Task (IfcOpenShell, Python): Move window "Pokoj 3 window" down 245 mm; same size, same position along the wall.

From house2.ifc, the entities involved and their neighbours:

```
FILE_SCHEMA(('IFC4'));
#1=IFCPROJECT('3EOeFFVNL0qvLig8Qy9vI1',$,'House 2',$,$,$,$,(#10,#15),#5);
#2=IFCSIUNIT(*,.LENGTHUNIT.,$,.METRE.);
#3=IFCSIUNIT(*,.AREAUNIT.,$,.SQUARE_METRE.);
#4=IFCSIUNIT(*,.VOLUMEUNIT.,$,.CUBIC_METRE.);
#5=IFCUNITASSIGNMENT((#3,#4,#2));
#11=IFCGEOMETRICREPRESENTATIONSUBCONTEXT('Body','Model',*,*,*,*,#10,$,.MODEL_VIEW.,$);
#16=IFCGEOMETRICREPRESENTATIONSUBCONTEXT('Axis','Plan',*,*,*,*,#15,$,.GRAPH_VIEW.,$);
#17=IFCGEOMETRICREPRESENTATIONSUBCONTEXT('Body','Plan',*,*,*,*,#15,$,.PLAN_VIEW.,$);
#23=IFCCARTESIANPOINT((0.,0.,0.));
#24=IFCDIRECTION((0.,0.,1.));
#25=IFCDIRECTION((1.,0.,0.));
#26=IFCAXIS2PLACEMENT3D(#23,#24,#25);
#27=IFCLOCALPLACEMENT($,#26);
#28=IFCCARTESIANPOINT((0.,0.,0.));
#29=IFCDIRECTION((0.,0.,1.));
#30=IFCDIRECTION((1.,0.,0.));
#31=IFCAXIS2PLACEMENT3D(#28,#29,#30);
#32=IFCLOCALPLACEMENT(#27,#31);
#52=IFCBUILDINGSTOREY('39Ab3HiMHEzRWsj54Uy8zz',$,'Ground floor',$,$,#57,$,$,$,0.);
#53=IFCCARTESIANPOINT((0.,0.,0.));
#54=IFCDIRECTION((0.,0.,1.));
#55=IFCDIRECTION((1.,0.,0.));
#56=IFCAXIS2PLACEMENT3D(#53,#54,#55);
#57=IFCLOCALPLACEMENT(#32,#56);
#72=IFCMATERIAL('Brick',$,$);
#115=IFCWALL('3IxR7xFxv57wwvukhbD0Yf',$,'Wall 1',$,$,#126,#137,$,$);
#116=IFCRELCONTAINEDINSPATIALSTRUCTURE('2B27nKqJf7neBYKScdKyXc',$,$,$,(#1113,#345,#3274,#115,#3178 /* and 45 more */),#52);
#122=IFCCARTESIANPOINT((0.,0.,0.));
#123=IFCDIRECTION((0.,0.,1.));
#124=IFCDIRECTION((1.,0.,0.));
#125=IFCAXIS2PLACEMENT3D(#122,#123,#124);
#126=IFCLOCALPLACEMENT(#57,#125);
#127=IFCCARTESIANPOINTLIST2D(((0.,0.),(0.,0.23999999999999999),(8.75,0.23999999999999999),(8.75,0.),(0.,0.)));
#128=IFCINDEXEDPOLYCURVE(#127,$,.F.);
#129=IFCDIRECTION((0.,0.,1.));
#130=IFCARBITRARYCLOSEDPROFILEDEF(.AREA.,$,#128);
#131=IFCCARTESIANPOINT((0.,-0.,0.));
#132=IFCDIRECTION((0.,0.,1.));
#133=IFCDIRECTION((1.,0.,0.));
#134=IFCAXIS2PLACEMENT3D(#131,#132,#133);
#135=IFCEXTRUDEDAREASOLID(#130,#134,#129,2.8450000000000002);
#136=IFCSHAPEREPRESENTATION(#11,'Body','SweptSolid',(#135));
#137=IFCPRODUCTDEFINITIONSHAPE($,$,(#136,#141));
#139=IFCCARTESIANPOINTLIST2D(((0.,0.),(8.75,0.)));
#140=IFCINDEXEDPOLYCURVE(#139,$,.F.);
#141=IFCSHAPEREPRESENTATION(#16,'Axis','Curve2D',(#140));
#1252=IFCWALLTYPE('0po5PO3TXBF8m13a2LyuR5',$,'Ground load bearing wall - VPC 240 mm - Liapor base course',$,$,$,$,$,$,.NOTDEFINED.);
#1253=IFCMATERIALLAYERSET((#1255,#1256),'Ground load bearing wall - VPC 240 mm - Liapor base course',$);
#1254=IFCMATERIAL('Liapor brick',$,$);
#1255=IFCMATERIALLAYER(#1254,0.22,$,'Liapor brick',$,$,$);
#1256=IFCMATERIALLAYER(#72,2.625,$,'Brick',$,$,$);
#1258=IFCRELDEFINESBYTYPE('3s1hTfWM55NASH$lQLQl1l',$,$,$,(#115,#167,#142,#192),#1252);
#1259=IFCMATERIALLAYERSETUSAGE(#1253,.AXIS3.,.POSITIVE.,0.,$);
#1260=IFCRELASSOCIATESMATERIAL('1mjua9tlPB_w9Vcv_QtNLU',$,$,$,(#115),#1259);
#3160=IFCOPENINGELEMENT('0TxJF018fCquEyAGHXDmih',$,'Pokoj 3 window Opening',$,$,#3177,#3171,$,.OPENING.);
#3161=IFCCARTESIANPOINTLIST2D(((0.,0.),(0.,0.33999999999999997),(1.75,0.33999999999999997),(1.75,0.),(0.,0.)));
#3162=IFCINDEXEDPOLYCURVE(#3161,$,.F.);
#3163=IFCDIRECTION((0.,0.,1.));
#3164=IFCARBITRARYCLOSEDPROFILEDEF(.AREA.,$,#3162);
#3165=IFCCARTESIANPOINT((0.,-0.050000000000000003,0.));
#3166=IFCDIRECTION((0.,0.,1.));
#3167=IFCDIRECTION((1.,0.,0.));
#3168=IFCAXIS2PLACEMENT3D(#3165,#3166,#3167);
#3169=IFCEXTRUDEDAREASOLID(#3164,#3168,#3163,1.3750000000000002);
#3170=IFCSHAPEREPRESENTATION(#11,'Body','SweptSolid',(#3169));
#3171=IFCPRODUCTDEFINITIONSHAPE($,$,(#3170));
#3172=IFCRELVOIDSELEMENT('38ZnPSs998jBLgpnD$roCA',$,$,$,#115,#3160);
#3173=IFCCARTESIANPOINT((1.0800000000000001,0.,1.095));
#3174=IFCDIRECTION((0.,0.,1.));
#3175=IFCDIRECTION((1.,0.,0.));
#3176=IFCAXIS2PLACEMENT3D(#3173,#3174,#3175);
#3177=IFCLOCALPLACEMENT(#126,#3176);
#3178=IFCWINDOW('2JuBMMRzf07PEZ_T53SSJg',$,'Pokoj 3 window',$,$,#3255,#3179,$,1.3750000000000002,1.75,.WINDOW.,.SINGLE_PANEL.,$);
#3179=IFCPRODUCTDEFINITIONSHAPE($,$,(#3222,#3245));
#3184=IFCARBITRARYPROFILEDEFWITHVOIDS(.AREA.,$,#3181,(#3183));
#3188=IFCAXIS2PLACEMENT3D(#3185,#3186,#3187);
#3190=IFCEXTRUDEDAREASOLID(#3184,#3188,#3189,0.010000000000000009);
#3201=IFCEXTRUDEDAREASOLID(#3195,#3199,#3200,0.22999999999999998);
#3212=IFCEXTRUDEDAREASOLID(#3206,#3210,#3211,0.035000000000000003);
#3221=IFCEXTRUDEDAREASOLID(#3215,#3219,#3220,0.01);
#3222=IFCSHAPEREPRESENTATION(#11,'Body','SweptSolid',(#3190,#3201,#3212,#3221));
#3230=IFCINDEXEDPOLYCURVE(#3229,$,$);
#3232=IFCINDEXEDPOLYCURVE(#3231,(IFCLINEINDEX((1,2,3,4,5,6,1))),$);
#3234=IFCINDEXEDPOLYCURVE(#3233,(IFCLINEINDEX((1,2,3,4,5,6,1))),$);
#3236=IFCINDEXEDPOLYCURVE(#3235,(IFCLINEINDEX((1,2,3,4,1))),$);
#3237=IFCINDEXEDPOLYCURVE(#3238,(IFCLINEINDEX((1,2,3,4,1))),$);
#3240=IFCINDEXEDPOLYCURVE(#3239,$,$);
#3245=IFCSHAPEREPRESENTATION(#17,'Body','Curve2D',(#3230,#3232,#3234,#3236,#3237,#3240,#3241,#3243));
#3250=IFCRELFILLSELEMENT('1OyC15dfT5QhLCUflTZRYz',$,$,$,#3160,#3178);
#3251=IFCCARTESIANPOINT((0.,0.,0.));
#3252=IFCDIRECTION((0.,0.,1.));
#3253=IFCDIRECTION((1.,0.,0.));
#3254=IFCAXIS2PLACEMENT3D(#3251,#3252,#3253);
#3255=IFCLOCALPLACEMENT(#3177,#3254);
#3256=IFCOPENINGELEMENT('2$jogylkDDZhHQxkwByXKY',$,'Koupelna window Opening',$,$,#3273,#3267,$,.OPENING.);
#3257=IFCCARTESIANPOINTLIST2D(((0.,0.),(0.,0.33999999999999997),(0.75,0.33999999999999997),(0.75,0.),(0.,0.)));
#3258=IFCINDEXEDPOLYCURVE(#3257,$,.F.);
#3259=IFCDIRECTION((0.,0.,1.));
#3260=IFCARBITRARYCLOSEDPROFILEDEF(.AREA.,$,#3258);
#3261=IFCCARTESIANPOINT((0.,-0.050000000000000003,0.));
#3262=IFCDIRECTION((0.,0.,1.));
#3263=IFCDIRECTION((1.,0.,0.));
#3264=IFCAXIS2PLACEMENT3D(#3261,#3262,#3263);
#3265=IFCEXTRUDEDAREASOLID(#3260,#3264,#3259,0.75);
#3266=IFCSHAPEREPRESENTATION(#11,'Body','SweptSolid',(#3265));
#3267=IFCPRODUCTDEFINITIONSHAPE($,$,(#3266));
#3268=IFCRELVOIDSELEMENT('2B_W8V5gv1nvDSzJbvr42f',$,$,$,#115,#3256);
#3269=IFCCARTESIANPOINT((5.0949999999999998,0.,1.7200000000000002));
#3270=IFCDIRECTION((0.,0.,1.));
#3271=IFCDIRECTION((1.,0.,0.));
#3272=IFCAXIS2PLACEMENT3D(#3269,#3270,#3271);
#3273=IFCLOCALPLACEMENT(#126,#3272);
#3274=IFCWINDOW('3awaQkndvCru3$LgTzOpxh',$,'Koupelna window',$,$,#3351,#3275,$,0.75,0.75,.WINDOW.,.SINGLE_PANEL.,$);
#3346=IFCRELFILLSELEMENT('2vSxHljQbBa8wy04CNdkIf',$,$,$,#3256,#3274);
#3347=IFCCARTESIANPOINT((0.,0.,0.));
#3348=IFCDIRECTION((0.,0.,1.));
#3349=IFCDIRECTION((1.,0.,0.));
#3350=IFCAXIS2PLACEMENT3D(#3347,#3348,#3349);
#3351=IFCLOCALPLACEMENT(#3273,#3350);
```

```python
import numpy as np
import ifcopenshell
import ifcopenshell.api.geometry
import ifcopenshell.util.placement
import ifcopenshell.util.unit

model = ifcopenshell.open("house2.ifc")
unit_scale = ifcopenshell.util.unit.calculate_unit_scale(model)

window = model.by_guid("2JuBMMRzf07PEZ_T53SSJg")
opening = window.FillsVoids[0].RelatingOpeningElement
dz = -0.245 / unit_scale

shift = np.array([0.0, 0.0, dz])
# The window is placed relative to its opening, so it follows when the opening moves.
matrix = ifcopenshell.util.placement.get_local_placement(opening.ObjectPlacement)
matrix[:3, 3] += shift
ifcopenshell.api.geometry.edit_object_placement(
    model, product=opening, matrix=matrix, is_si=False, should_transform_children=True
)

print(f"moved by {dz * unit_scale:+.3f} m")

model.write("house2_updated.ifc")
```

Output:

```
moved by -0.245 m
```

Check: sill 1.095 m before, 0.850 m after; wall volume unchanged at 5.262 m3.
